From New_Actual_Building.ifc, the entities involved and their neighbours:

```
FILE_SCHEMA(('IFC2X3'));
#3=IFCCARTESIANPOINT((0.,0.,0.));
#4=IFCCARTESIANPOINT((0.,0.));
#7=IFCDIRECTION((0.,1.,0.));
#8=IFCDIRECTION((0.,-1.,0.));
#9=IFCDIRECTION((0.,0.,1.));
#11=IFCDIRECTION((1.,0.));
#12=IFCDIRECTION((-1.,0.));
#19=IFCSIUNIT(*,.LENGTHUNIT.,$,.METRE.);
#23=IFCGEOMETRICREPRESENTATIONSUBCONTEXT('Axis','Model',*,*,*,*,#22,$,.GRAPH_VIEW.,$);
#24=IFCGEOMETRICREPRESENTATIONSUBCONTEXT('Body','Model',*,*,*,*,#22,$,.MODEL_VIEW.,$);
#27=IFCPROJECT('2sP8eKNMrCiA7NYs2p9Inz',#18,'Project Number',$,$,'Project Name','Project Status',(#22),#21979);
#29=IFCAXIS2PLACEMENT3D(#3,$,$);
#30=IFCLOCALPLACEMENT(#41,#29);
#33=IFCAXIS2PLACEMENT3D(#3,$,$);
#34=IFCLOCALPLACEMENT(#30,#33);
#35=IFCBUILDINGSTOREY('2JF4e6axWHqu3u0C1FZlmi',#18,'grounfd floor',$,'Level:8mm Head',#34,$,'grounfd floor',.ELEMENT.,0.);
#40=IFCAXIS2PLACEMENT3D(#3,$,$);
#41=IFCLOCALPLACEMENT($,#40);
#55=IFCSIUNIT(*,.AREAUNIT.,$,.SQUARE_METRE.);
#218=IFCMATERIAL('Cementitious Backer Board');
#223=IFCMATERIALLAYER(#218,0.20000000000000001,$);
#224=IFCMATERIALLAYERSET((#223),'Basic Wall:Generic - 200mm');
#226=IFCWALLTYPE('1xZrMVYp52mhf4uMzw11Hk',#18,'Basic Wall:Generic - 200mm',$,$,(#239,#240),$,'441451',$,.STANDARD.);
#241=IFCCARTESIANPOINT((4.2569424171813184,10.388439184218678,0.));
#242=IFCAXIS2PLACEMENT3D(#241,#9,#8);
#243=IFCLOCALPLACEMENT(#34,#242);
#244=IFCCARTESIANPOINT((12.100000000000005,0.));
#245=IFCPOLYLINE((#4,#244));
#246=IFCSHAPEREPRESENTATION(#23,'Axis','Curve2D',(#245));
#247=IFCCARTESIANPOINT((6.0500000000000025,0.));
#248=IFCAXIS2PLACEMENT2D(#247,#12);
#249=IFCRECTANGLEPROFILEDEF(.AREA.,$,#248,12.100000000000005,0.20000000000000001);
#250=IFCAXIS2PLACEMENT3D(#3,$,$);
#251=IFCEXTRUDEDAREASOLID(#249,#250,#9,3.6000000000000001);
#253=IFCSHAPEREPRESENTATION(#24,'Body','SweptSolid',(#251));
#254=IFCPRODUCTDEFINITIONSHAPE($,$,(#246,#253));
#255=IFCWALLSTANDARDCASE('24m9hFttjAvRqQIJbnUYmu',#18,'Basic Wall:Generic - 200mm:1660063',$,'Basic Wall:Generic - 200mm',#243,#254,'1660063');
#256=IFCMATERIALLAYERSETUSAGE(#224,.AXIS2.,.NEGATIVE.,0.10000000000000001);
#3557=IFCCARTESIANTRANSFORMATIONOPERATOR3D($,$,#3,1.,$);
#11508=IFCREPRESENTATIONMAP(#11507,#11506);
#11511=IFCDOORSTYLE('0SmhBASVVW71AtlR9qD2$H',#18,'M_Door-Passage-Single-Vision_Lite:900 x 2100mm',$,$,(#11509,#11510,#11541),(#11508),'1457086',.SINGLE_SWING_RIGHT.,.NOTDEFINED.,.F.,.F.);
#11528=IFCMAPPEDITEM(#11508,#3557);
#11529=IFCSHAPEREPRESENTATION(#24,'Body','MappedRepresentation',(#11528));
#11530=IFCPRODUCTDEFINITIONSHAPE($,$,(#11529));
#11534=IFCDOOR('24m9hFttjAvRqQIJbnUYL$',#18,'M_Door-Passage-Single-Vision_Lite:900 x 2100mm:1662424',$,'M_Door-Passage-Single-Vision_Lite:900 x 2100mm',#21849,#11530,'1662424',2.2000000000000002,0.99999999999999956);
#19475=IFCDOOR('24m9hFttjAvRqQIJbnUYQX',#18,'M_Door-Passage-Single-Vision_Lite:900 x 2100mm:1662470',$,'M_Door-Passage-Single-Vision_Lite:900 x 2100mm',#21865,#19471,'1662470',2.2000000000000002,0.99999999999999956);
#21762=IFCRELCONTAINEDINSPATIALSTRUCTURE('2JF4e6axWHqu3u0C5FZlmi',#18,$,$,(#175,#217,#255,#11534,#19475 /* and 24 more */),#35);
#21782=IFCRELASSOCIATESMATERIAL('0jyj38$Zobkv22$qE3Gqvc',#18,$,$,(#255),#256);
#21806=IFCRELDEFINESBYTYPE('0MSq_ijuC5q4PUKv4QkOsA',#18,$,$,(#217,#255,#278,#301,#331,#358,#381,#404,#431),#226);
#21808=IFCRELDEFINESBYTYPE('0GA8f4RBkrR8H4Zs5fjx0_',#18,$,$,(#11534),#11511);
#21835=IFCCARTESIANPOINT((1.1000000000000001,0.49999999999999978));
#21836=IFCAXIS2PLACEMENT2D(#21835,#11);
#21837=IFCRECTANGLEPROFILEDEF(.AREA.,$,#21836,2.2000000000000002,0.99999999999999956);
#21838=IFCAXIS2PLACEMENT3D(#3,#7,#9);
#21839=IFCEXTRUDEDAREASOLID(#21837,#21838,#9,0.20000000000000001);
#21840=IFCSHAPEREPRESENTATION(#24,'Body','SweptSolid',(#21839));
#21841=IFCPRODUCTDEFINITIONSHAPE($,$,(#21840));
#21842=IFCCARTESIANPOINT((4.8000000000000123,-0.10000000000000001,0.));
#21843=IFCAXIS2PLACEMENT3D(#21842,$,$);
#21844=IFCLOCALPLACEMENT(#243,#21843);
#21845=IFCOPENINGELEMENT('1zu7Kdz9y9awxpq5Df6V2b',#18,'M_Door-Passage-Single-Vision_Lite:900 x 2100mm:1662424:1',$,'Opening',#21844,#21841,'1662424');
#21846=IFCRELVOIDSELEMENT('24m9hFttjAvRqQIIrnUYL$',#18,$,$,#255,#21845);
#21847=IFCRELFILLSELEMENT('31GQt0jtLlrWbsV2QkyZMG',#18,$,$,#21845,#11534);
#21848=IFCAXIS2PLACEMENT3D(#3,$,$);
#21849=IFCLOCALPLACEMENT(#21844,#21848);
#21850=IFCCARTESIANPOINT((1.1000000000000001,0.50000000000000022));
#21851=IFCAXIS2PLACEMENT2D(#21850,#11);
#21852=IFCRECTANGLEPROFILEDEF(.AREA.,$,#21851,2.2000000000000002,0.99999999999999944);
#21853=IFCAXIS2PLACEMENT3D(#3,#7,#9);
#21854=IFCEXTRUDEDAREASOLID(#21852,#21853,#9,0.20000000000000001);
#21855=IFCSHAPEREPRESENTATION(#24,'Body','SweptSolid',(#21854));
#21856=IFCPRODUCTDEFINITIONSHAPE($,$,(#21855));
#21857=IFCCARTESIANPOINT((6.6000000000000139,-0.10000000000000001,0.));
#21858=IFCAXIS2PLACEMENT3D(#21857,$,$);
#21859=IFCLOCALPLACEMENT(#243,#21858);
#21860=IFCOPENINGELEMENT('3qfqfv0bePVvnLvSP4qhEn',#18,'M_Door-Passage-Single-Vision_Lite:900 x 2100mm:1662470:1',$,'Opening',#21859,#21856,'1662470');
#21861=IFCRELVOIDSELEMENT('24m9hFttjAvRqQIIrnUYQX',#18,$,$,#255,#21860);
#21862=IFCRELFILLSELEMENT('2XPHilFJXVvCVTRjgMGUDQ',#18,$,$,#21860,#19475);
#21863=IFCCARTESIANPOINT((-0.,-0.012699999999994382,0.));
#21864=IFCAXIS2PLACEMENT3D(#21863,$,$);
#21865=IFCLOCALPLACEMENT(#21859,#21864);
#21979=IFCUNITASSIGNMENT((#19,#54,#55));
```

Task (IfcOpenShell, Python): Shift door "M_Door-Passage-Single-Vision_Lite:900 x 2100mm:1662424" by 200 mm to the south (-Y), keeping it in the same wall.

```python
import ifcopenshell
import ifcopenshell.api.geometry
import ifcopenshell.util.placement
import ifcopenshell.util.unit

model = ifcopenshell.open("New_Actual_Building.ifc")
unit_scale = ifcopenshell.util.unit.calculate_unit_scale(model)

door = model.by_id(11534)
opening = door.FillsVoids[0].RelatingOpeningElement
wall = opening.VoidsElements[0].RelatingBuildingElement

wall_matrix = ifcopenshell.util.placement.get_local_placement(wall.ObjectPlacement)
shift = wall_matrix[:3, 0] * 0.2 / unit_scale
before = ifcopenshell.util.placement.get_local_placement(door.ObjectPlacement)[:3, 3].copy()

# The door is placed relative to its opening, so it follows when the opening moves.
matrix = ifcopenshell.util.placement.get_local_placement(opening.ObjectPlacement)
matrix[:3, 3] += shift
ifcopenshell.api.geometry.edit_object_placement(
    model, product=opening, matrix=matrix, is_si=False, should_transform_children=True
)

after = ifcopenshell.util.placement.get_local_placement(door.ObjectPlacement)[:3, 3]
print("door moved by", (after - before).round(3) + 0.0)

model.write("New_Actual_Building_v2.ifc")
```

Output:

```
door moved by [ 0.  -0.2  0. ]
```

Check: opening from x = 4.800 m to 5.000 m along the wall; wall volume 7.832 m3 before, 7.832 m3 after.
